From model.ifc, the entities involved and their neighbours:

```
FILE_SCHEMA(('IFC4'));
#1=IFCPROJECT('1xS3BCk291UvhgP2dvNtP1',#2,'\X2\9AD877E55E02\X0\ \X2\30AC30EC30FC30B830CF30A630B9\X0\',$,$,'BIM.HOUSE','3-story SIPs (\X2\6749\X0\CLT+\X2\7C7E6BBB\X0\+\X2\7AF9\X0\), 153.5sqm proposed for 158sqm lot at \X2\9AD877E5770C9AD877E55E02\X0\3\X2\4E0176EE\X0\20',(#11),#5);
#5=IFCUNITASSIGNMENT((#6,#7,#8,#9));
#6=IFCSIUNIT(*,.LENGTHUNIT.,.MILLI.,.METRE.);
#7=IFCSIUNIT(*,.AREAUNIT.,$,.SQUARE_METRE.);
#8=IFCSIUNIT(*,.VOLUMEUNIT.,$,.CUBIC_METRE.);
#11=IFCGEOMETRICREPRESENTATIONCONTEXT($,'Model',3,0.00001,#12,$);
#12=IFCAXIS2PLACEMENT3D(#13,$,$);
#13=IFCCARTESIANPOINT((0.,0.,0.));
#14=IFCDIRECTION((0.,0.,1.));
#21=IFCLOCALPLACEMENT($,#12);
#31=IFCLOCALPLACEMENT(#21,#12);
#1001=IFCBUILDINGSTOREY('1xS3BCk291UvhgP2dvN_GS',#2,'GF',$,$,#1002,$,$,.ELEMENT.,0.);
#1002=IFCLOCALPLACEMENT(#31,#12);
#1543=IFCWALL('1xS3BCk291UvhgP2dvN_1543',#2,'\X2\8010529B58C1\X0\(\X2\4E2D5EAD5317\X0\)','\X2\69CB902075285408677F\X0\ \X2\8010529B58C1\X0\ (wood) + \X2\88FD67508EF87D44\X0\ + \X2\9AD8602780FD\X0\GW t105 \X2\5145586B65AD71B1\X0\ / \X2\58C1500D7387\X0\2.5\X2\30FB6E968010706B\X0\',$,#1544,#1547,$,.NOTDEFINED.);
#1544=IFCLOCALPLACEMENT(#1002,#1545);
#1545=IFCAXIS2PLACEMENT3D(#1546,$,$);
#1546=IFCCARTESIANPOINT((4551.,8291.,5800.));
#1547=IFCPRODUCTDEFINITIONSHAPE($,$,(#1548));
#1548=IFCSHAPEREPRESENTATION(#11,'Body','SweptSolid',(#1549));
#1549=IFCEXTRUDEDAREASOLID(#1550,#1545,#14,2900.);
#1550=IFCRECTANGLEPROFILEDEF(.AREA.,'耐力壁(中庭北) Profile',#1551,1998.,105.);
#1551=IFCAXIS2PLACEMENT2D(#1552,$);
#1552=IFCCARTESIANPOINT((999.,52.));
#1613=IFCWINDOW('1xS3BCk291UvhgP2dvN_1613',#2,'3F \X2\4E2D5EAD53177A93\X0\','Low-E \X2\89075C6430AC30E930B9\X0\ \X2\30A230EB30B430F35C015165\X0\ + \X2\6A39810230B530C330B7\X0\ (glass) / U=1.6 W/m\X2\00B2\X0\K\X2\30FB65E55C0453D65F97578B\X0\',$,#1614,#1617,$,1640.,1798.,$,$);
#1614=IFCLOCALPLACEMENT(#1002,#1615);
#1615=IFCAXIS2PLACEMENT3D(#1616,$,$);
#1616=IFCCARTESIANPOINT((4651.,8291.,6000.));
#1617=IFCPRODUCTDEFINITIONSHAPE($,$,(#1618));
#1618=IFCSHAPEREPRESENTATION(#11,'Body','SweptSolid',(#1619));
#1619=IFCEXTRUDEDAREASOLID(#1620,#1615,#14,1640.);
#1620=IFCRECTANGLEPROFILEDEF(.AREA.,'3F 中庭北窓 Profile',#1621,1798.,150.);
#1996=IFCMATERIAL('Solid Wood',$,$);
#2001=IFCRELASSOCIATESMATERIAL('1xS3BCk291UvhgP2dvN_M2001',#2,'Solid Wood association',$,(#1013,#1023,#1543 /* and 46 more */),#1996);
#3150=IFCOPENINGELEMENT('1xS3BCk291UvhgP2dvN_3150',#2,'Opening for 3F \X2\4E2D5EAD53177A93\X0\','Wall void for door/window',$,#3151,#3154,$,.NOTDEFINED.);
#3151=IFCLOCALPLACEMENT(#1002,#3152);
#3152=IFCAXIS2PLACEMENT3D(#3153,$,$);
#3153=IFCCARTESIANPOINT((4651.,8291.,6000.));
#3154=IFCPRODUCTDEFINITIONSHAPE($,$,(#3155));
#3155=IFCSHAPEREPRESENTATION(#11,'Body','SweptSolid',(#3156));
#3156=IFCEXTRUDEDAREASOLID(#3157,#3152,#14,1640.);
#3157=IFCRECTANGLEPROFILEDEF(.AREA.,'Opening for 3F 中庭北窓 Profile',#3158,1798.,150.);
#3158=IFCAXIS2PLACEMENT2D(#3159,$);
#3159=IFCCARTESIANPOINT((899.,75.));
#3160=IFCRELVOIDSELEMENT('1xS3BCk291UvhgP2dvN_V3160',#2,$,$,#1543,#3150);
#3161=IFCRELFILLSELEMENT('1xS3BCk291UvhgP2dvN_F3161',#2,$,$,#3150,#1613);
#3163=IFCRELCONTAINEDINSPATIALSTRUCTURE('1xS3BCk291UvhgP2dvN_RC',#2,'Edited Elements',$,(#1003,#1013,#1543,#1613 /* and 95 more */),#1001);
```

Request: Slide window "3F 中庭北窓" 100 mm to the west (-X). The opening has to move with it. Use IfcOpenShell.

```python
import ifcopenshell
import ifcopenshell.api.geometry
import ifcopenshell.util.placement

model = ifcopenshell.open("model.ifc")

window = model.by_guid("1xS3BCk291UvhgP2dvN_1613")
opening = window.FillsVoids[0].RelatingOpeningElement
wall = opening.VoidsElements[0].RelatingBuildingElement

wall_matrix = ifcopenshell.util.placement.get_local_placement(wall.ObjectPlacement)
shift = wall_matrix[:3, 0] * -100.0
before = ifcopenshell.util.placement.get_local_placement(window.ObjectPlacement)[:3, 3].copy()

# The window is not placed relative to its opening, so move both.
for product in (opening, window):
    matrix = ifcopenshell.util.placement.get_local_placement(product.ObjectPlacement)
    matrix[:3, 3] += shift
    ifcopenshell.api.geometry.edit_object_placement(model, product=product, matrix=matrix, is_si=False)

after = ifcopenshell.util.placement.get_local_placement(window.ObjectPlacement)[:3, 3]
print("window moved by", (after - before).round(3) + 0.0)

model.write("model_rev.ifc")
```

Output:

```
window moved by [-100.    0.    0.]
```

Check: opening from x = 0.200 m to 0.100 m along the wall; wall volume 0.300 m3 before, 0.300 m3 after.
